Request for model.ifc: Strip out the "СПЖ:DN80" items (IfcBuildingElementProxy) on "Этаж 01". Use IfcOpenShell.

First a look at what the model holds.

```python
import ifcopenshell
import ifcopenshell.util.element

model = ifcopenshell.open("model.ifc")
print(model.schema)
storey = next(s for s in model.by_type("IfcBuildingStorey") if s.Name == "Этаж 01")
proxies = [e for e in ifcopenshell.util.element.get_decomposition(storey) if e.is_a("IfcBuildingElementProxy")]
seen = {}
for e in proxies:
    element_type = ifcopenshell.util.element.get_type(e)
    name = element_type.Name if element_type not in (None, e) else None
    seen[name] = seen.get(name, 0) + 1
for name, count in sorted(seen.items(), key=str):
    print(count, "x", name)
```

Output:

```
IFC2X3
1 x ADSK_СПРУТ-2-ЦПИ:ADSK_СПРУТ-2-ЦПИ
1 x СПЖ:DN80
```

```python
import ifcopenshell
import ifcopenshell.api.root
import ifcopenshell.util.element

model = ifcopenshell.open("model.ifc")

storey = next(s for s in model.by_type("IfcBuildingStorey") if s.Name == "Этаж 01")
proxies = [e for e in ifcopenshell.util.element.get_decomposition(storey) if e.is_a("IfcBuildingElementProxy")]
targets = [e for e in proxies if (t := ifcopenshell.util.element.get_type(e)) not in (None, e) and t.Name == "СПЖ:DN80"]

for e in targets:
    ifcopenshell.api.root.remove_product(model, product=e)
print(len(targets), "removed")

model.write("model-out.ifc")
```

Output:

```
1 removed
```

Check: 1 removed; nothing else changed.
